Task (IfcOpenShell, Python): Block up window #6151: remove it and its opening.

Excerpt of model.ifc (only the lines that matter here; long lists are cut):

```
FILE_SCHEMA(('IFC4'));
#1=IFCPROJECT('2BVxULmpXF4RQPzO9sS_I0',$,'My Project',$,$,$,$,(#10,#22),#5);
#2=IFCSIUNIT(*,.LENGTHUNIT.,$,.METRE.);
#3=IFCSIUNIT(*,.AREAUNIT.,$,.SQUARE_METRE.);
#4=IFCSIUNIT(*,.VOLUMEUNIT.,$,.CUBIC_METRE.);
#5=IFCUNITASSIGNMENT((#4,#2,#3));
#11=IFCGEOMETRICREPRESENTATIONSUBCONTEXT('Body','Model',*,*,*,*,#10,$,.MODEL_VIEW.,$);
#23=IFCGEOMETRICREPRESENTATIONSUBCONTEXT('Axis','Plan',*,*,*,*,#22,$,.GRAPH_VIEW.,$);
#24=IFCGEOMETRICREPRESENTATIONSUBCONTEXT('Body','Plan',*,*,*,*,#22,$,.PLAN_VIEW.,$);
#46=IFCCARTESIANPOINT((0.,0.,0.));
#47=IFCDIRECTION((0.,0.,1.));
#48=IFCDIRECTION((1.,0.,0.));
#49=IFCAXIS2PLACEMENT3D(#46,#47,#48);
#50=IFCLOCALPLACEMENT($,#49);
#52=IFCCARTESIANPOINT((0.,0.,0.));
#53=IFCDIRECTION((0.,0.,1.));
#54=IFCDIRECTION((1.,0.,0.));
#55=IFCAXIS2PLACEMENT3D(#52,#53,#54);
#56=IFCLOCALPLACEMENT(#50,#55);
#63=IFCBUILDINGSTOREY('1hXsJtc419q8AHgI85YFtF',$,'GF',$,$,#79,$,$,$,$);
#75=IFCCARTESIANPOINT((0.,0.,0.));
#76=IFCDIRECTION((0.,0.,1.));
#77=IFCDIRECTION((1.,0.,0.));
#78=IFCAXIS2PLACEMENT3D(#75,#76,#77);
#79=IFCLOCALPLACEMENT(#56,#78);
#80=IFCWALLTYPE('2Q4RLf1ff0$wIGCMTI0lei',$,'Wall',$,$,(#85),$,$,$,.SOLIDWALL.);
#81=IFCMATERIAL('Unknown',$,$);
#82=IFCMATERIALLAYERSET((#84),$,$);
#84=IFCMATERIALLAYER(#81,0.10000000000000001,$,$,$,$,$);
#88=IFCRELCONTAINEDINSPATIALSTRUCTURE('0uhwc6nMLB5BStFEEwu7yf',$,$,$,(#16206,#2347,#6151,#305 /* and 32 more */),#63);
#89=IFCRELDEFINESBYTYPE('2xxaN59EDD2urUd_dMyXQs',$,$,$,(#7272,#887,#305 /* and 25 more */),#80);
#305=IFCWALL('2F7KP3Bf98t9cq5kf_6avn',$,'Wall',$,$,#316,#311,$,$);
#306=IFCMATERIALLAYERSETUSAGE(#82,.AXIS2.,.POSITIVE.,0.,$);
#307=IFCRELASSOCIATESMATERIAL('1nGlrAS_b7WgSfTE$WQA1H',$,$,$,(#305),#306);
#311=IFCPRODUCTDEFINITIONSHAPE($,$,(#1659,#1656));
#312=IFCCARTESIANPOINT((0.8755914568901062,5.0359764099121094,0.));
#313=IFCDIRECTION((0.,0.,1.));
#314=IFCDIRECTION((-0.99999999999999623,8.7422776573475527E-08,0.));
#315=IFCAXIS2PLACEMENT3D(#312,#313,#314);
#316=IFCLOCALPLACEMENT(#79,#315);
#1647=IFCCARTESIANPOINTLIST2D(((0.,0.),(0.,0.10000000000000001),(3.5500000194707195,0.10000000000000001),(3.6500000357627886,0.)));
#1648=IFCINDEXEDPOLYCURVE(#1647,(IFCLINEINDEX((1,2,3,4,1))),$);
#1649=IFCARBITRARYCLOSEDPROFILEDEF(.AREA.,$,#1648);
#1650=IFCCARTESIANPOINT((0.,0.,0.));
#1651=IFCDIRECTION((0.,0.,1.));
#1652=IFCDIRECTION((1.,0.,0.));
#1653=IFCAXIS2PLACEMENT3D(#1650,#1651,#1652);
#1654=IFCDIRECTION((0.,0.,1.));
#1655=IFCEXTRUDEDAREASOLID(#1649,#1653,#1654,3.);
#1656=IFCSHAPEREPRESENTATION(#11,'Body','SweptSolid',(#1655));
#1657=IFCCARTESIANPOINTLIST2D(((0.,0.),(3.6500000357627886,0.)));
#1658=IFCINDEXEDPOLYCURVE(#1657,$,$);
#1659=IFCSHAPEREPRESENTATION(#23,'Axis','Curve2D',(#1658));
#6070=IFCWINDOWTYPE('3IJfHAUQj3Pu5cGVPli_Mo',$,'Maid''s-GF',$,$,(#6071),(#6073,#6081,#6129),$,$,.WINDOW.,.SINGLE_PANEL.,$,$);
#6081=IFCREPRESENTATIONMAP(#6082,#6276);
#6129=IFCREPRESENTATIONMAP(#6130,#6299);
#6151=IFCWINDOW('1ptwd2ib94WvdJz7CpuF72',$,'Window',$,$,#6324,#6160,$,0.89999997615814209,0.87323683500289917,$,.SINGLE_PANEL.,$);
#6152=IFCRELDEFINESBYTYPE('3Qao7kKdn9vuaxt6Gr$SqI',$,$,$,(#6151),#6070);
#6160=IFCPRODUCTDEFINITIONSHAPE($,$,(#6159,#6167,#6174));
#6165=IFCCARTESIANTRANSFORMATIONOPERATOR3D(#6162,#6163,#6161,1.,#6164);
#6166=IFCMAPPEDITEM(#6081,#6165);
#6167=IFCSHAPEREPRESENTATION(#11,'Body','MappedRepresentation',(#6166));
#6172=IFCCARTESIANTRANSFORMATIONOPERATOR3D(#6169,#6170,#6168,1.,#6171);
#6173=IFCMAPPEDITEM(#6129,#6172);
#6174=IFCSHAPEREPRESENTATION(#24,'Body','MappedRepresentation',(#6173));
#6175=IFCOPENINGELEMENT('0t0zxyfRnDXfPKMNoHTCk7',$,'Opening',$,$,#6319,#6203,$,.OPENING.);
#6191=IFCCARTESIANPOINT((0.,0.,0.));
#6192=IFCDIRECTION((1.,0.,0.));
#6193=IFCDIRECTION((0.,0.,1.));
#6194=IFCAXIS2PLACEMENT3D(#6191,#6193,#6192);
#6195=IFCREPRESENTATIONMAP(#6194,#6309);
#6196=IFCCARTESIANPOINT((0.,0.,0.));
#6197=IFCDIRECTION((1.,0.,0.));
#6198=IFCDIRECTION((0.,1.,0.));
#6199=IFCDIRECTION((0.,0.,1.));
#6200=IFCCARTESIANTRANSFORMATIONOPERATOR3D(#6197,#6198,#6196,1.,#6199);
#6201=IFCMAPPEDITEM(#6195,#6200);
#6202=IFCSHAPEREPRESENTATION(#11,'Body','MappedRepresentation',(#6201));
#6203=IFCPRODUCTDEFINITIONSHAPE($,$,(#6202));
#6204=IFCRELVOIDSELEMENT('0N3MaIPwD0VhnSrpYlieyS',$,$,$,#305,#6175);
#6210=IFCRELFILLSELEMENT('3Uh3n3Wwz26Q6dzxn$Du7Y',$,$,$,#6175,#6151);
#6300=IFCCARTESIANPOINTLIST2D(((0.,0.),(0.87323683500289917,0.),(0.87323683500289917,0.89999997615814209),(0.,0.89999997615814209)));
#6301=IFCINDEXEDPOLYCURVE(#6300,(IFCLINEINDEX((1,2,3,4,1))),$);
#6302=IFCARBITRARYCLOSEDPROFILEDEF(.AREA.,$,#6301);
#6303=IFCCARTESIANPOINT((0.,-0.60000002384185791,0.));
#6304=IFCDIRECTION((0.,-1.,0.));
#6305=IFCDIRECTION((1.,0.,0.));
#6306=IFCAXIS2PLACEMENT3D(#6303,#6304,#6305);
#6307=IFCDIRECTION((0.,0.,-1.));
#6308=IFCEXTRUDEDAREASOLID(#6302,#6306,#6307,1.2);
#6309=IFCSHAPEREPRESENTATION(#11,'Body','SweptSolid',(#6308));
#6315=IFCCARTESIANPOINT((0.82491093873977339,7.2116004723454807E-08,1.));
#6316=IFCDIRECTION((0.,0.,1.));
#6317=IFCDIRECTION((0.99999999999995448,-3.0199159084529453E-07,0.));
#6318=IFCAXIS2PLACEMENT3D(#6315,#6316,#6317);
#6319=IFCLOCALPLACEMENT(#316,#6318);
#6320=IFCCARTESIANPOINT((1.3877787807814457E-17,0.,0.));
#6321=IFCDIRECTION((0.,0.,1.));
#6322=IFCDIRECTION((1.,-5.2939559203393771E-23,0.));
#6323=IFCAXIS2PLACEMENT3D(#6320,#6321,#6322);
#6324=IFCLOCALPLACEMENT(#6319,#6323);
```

```python
import ifcopenshell
import ifcopenshell.api.feature
import ifcopenshell.api.root
import ifcopenshell.geom
import ifcopenshell.util.shape

model = ifcopenshell.open("model.ifc")
settings = ifcopenshell.geom.settings()


def volume(element):
    """Net volume in cubic metres, openings subtracted."""
    shape = ifcopenshell.geom.create_shape(settings, element)
    return ifcopenshell.util.shape.get_volume(shape.geometry)


window = model.by_id(6151)
opening = window.FillsVoids[0].RelatingOpeningElement
wall = opening.VoidsElements[0].RelatingBuildingElement
before = volume(wall)

ifcopenshell.api.root.remove_product(model, product=window)
ifcopenshell.api.feature.remove_feature(model, feature=opening)

after = volume(wall)

print(f"wall volume {before:.3f} -> {after:.3f} m3")

model.write("model-out.ifc")
```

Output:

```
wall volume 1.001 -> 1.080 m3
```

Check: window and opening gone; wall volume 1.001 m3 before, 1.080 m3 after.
